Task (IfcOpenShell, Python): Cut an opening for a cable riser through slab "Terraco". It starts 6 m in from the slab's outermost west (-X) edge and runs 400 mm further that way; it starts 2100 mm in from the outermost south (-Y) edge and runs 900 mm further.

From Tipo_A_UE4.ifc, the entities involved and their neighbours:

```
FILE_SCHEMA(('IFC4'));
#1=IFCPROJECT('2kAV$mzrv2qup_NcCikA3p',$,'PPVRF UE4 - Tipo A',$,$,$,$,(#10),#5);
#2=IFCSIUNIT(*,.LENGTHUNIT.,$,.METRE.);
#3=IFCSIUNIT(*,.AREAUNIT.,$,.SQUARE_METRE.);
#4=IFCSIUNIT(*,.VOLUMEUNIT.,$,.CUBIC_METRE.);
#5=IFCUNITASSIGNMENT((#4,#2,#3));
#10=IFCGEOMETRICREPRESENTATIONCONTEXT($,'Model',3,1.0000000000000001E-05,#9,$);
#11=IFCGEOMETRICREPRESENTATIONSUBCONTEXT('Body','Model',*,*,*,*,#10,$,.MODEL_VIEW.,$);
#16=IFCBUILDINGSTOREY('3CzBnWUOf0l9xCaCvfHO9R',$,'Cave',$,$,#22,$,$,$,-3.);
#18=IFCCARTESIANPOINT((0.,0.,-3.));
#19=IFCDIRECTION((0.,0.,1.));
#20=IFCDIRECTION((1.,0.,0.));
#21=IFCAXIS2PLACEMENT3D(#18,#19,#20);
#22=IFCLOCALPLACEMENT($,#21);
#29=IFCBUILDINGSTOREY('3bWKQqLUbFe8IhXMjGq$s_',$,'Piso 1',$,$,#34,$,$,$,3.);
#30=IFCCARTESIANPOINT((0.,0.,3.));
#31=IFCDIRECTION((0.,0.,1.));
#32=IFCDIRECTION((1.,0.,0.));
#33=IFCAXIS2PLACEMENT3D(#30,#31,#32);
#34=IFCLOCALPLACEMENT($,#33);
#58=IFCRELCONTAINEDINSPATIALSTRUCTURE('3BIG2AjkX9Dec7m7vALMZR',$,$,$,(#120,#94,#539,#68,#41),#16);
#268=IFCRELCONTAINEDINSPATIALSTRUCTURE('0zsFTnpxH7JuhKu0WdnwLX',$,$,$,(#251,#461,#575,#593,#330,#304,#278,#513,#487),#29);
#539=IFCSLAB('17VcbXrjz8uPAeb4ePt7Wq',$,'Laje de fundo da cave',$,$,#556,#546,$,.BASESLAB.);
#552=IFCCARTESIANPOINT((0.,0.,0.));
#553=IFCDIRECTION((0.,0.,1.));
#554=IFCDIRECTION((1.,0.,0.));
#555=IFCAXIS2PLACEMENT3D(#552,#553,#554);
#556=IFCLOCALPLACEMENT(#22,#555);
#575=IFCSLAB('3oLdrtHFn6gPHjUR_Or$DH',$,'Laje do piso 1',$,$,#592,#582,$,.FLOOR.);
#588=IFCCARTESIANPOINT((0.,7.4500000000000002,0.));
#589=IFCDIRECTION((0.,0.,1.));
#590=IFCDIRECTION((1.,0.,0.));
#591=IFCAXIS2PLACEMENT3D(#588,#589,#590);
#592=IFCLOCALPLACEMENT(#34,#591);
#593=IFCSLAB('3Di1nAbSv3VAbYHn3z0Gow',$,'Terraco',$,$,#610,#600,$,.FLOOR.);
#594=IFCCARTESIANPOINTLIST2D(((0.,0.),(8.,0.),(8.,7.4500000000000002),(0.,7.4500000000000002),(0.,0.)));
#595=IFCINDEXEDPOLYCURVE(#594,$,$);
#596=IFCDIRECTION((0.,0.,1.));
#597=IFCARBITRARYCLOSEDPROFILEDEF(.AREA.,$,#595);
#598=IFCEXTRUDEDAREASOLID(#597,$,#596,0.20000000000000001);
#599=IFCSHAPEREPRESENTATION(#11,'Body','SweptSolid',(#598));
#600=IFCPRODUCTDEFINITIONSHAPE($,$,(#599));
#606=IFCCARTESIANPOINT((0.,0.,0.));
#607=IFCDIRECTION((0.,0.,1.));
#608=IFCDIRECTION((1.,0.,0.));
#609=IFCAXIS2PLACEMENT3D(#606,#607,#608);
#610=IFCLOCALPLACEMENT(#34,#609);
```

```python
import numpy as np
import ifcopenshell
import ifcopenshell.api.feature
import ifcopenshell.api.geometry
import ifcopenshell.api.root
import ifcopenshell.geom
import ifcopenshell.util.placement
import ifcopenshell.util.representation
import ifcopenshell.util.shape
import ifcopenshell.util.unit

model = ifcopenshell.open("Tipo_A_UE4.ifc")
unit_scale = ifcopenshell.util.unit.calculate_unit_scale(model)
settings = ifcopenshell.geom.settings()


def volume(element):
    """Net volume in cubic metres, openings subtracted."""
    shape = ifcopenshell.geom.create_shape(settings, element)
    return ifcopenshell.util.shape.get_volume(shape.geometry)


slab = model.by_id(593)
before = volume(slab)

# Extent in the slab's own axes, in metres. The edges named are its -X and -Y sides.
slab_shape = ifcopenshell.geom.create_shape(settings, slab)
vertices = ifcopenshell.util.shape.get_vertices(slab_shape.geometry)
x_min, y_min, bottom = vertices.min(axis=0)
top = vertices[:, 2].max()

opening = ifcopenshell.api.root.create_entity(model, ifc_class="IfcOpeningElement", name="Cable riser opening", predefined_type="OPENING")
context = ifcopenshell.util.representation.get_context(model, "Model", "Body", "MODEL_VIEW")
width, depth = 0.4, 0.9
outline = [(0.0, 0.0), (width, 0.0), (width, depth), (0.0, depth), (0.0, 0.0)]
# Overshoot both faces by 50 mm so the cut is clean.
shape = ifcopenshell.api.geometry.add_slab_representation(
    model, context=context, depth=top - bottom + 0.1, polyline=outline
)
ifcopenshell.api.geometry.assign_representation(model, product=opening, representation=shape)

matrix = ifcopenshell.util.placement.get_local_placement(slab.ObjectPlacement)
matrix[:, 3] = matrix @ np.append(np.array([x_min + 6, y_min + 2.1, bottom - 0.05]) / unit_scale, 1.0)
ifcopenshell.api.geometry.edit_object_placement(model, product=opening, matrix=matrix, is_si=False)
ifcopenshell.api.feature.add_feature(model, feature=opening, element=slab)

after = volume(slab)

print(f"slab volume {before:.3f} -> {after:.3f} m3")

model.write("Tipo_A_UE4-out.ifc")
```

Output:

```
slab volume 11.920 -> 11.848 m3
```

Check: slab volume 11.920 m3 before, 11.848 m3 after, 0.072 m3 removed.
